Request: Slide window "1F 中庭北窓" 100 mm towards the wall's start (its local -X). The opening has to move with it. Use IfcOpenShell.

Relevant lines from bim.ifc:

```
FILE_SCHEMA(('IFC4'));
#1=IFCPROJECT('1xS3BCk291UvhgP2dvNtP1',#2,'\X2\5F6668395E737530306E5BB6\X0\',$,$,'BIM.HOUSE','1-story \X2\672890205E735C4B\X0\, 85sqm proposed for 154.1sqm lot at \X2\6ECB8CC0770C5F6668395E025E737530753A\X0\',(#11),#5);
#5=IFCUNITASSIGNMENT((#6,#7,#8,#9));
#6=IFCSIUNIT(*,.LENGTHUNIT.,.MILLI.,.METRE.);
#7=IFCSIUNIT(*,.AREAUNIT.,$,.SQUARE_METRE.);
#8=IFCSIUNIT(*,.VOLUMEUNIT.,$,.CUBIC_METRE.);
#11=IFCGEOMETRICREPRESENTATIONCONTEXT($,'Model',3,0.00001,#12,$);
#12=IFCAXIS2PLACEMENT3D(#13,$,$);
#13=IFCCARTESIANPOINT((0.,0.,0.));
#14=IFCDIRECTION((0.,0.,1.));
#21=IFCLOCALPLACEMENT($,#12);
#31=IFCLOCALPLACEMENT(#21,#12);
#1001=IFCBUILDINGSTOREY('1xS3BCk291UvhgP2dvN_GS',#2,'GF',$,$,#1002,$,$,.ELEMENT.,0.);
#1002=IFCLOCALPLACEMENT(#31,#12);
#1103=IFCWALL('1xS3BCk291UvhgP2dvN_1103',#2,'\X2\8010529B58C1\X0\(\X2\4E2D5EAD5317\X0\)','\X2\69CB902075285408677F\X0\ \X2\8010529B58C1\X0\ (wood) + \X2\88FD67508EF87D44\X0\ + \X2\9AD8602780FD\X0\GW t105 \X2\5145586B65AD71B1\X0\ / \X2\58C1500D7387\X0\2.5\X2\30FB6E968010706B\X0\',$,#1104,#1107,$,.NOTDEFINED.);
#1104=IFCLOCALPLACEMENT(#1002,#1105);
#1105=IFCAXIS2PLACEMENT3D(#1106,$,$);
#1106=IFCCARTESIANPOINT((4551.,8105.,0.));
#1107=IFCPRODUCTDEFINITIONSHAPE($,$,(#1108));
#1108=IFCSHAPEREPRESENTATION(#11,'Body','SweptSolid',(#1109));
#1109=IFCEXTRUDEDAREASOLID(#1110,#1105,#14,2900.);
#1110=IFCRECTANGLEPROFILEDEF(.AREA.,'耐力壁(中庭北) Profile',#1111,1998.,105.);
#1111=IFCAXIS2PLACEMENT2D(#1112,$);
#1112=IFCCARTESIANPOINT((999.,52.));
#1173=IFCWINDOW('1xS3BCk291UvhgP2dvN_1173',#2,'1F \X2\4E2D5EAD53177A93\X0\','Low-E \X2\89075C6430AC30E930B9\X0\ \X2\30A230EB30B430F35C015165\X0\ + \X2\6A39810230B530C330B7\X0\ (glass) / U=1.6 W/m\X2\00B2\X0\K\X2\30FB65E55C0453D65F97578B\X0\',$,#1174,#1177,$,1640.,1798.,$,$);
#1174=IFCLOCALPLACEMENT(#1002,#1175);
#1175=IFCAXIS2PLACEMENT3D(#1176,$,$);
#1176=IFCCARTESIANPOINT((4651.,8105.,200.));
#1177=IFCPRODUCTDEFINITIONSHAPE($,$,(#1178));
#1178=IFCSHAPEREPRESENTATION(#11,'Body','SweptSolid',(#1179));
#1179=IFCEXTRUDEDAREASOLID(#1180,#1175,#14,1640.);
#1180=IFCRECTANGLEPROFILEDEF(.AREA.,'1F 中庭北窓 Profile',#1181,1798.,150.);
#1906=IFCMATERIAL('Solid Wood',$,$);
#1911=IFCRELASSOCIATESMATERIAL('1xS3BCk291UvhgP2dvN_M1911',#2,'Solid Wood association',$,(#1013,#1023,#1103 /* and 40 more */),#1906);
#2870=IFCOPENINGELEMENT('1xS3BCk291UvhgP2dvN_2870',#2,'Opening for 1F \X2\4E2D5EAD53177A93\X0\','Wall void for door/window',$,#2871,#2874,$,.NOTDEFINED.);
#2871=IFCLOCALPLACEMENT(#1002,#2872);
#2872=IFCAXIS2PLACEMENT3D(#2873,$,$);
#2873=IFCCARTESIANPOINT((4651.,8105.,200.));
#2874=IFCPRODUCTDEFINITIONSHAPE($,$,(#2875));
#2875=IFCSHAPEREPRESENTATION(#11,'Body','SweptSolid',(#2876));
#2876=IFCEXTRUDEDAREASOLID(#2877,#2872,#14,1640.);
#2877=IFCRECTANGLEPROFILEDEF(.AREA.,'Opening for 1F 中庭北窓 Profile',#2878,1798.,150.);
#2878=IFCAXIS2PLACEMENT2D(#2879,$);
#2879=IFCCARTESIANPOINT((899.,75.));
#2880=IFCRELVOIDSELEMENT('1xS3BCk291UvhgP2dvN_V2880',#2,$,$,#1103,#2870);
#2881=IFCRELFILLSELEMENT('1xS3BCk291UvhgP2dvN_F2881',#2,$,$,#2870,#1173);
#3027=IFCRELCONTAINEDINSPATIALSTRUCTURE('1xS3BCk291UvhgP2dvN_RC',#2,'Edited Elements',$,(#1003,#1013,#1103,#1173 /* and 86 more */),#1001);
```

```python
import ifcopenshell
import ifcopenshell.api.geometry
import ifcopenshell.util.placement

model = ifcopenshell.open("bim.ifc")

window = model.by_id(1173)
opening = window.FillsVoids[0].RelatingOpeningElement
wall = opening.VoidsElements[0].RelatingBuildingElement

wall_matrix = ifcopenshell.util.placement.get_local_placement(wall.ObjectPlacement)
shift = wall_matrix[:3, 0] * -100.0
before = ifcopenshell.util.placement.get_local_placement(window.ObjectPlacement)[:3, 3].copy()

# The window is not placed relative to its opening, so move both.
for product in (opening, window):
    matrix = ifcopenshell.util.placement.get_local_placement(product.ObjectPlacement)
    matrix[:3, 3] += shift
    ifcopenshell.api.geometry.edit_object_placement(model, product=product, matrix=matrix, is_si=False)

after = ifcopenshell.util.placement.get_local_placement(window.ObjectPlacement)[:3, 3]
print("window moved by", (after - before).round(3) + 0.0)

model.write("bim-out.ifc")
```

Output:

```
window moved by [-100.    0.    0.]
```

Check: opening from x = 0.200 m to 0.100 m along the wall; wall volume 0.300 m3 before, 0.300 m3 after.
